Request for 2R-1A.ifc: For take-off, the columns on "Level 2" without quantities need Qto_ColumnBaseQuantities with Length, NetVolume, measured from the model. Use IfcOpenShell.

First a look at what the model holds.

```python
import ifcopenshell
import ifcopenshell.util.element
import ifcopenshell.util.unit

model = ifcopenshell.open("2R-1A.ifc")
print(model.schema)
for unit_type in ("LENGTHUNIT", "AREAUNIT", "VOLUMEUNIT"):
    print(unit_type, ifcopenshell.util.unit.calculate_unit_scale(model, unit_type))
storey = next(s for s in model.by_type("IfcBuildingStorey") if s.Name == "Level 2")
columns = [e for e in ifcopenshell.util.element.get_decomposition(storey) if e.is_a("IfcColumn")]
for e in sorted(columns, key=lambda e: e.id()):
    print(e.id(), e.is_a(), e.Name, list(ifcopenshell.util.element.get_psets(e, qtos_only=True)), sep=" | ")
```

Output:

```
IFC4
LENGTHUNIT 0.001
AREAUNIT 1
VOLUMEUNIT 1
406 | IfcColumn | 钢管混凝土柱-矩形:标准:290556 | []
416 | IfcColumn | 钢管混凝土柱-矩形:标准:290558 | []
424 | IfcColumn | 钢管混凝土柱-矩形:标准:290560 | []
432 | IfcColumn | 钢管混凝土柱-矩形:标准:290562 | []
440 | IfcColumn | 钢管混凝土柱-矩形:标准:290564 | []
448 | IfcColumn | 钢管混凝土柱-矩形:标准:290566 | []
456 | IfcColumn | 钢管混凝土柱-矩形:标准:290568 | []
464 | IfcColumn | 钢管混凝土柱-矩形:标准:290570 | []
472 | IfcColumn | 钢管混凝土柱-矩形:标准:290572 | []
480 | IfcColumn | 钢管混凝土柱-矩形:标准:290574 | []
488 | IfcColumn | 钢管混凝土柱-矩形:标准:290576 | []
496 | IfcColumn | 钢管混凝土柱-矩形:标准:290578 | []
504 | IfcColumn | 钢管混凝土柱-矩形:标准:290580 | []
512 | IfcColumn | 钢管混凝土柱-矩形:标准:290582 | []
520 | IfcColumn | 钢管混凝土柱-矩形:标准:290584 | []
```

```python
import ifcopenshell
import ifcopenshell.api.pset
import ifcopenshell.geom
import ifcopenshell.util.element
import ifcopenshell.util.shape
import ifcopenshell.util.unit

model = ifcopenshell.open("2R-1A.ifc")
unit_scale = ifcopenshell.util.unit.calculate_unit_scale(model)
volume_scale = ifcopenshell.util.unit.calculate_unit_scale(model, "VOLUMEUNIT")
settings = ifcopenshell.geom.settings()

storey = next(s for s in model.by_type("IfcBuildingStorey") if s.Name == "Level 2")
columns = [e for e in ifcopenshell.util.element.get_decomposition(storey) if e.is_a("IfcColumn")]

for e in sorted(columns, key=lambda e: e.id()):
    if ifcopenshell.util.element.get_psets(e, qtos_only=True, should_inherit=False):
        continue
    # Geometry comes back in metres, in the element's own axes.
    shape = ifcopenshell.geom.create_shape(settings, e)
    values = {
        "Length": ifcopenshell.util.shape.get_z(shape.geometry) / unit_scale,
        "NetVolume": ifcopenshell.util.shape.get_volume(shape.geometry) / volume_scale,
    }
    qto = ifcopenshell.api.pset.add_qto(model, product=e, name="Qto_ColumnBaseQuantities")
    ifcopenshell.api.pset.edit_qto(model, qto=qto, properties=values)
    print(e.id(), {k: round(v, 3) for k, v in values.items()})

model.write("2R-1A-out.ifc")
```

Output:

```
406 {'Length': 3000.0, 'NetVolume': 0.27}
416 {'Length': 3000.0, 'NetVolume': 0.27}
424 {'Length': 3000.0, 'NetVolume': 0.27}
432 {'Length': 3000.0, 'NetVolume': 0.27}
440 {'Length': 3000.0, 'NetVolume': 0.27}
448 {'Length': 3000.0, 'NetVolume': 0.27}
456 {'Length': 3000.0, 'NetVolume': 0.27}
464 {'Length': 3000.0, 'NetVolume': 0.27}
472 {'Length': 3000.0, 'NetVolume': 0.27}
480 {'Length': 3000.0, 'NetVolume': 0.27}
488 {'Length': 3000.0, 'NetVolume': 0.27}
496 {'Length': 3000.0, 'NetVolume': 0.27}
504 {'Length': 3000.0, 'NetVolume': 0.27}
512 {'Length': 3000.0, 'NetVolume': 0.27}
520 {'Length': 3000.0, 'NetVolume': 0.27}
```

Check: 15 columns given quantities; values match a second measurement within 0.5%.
